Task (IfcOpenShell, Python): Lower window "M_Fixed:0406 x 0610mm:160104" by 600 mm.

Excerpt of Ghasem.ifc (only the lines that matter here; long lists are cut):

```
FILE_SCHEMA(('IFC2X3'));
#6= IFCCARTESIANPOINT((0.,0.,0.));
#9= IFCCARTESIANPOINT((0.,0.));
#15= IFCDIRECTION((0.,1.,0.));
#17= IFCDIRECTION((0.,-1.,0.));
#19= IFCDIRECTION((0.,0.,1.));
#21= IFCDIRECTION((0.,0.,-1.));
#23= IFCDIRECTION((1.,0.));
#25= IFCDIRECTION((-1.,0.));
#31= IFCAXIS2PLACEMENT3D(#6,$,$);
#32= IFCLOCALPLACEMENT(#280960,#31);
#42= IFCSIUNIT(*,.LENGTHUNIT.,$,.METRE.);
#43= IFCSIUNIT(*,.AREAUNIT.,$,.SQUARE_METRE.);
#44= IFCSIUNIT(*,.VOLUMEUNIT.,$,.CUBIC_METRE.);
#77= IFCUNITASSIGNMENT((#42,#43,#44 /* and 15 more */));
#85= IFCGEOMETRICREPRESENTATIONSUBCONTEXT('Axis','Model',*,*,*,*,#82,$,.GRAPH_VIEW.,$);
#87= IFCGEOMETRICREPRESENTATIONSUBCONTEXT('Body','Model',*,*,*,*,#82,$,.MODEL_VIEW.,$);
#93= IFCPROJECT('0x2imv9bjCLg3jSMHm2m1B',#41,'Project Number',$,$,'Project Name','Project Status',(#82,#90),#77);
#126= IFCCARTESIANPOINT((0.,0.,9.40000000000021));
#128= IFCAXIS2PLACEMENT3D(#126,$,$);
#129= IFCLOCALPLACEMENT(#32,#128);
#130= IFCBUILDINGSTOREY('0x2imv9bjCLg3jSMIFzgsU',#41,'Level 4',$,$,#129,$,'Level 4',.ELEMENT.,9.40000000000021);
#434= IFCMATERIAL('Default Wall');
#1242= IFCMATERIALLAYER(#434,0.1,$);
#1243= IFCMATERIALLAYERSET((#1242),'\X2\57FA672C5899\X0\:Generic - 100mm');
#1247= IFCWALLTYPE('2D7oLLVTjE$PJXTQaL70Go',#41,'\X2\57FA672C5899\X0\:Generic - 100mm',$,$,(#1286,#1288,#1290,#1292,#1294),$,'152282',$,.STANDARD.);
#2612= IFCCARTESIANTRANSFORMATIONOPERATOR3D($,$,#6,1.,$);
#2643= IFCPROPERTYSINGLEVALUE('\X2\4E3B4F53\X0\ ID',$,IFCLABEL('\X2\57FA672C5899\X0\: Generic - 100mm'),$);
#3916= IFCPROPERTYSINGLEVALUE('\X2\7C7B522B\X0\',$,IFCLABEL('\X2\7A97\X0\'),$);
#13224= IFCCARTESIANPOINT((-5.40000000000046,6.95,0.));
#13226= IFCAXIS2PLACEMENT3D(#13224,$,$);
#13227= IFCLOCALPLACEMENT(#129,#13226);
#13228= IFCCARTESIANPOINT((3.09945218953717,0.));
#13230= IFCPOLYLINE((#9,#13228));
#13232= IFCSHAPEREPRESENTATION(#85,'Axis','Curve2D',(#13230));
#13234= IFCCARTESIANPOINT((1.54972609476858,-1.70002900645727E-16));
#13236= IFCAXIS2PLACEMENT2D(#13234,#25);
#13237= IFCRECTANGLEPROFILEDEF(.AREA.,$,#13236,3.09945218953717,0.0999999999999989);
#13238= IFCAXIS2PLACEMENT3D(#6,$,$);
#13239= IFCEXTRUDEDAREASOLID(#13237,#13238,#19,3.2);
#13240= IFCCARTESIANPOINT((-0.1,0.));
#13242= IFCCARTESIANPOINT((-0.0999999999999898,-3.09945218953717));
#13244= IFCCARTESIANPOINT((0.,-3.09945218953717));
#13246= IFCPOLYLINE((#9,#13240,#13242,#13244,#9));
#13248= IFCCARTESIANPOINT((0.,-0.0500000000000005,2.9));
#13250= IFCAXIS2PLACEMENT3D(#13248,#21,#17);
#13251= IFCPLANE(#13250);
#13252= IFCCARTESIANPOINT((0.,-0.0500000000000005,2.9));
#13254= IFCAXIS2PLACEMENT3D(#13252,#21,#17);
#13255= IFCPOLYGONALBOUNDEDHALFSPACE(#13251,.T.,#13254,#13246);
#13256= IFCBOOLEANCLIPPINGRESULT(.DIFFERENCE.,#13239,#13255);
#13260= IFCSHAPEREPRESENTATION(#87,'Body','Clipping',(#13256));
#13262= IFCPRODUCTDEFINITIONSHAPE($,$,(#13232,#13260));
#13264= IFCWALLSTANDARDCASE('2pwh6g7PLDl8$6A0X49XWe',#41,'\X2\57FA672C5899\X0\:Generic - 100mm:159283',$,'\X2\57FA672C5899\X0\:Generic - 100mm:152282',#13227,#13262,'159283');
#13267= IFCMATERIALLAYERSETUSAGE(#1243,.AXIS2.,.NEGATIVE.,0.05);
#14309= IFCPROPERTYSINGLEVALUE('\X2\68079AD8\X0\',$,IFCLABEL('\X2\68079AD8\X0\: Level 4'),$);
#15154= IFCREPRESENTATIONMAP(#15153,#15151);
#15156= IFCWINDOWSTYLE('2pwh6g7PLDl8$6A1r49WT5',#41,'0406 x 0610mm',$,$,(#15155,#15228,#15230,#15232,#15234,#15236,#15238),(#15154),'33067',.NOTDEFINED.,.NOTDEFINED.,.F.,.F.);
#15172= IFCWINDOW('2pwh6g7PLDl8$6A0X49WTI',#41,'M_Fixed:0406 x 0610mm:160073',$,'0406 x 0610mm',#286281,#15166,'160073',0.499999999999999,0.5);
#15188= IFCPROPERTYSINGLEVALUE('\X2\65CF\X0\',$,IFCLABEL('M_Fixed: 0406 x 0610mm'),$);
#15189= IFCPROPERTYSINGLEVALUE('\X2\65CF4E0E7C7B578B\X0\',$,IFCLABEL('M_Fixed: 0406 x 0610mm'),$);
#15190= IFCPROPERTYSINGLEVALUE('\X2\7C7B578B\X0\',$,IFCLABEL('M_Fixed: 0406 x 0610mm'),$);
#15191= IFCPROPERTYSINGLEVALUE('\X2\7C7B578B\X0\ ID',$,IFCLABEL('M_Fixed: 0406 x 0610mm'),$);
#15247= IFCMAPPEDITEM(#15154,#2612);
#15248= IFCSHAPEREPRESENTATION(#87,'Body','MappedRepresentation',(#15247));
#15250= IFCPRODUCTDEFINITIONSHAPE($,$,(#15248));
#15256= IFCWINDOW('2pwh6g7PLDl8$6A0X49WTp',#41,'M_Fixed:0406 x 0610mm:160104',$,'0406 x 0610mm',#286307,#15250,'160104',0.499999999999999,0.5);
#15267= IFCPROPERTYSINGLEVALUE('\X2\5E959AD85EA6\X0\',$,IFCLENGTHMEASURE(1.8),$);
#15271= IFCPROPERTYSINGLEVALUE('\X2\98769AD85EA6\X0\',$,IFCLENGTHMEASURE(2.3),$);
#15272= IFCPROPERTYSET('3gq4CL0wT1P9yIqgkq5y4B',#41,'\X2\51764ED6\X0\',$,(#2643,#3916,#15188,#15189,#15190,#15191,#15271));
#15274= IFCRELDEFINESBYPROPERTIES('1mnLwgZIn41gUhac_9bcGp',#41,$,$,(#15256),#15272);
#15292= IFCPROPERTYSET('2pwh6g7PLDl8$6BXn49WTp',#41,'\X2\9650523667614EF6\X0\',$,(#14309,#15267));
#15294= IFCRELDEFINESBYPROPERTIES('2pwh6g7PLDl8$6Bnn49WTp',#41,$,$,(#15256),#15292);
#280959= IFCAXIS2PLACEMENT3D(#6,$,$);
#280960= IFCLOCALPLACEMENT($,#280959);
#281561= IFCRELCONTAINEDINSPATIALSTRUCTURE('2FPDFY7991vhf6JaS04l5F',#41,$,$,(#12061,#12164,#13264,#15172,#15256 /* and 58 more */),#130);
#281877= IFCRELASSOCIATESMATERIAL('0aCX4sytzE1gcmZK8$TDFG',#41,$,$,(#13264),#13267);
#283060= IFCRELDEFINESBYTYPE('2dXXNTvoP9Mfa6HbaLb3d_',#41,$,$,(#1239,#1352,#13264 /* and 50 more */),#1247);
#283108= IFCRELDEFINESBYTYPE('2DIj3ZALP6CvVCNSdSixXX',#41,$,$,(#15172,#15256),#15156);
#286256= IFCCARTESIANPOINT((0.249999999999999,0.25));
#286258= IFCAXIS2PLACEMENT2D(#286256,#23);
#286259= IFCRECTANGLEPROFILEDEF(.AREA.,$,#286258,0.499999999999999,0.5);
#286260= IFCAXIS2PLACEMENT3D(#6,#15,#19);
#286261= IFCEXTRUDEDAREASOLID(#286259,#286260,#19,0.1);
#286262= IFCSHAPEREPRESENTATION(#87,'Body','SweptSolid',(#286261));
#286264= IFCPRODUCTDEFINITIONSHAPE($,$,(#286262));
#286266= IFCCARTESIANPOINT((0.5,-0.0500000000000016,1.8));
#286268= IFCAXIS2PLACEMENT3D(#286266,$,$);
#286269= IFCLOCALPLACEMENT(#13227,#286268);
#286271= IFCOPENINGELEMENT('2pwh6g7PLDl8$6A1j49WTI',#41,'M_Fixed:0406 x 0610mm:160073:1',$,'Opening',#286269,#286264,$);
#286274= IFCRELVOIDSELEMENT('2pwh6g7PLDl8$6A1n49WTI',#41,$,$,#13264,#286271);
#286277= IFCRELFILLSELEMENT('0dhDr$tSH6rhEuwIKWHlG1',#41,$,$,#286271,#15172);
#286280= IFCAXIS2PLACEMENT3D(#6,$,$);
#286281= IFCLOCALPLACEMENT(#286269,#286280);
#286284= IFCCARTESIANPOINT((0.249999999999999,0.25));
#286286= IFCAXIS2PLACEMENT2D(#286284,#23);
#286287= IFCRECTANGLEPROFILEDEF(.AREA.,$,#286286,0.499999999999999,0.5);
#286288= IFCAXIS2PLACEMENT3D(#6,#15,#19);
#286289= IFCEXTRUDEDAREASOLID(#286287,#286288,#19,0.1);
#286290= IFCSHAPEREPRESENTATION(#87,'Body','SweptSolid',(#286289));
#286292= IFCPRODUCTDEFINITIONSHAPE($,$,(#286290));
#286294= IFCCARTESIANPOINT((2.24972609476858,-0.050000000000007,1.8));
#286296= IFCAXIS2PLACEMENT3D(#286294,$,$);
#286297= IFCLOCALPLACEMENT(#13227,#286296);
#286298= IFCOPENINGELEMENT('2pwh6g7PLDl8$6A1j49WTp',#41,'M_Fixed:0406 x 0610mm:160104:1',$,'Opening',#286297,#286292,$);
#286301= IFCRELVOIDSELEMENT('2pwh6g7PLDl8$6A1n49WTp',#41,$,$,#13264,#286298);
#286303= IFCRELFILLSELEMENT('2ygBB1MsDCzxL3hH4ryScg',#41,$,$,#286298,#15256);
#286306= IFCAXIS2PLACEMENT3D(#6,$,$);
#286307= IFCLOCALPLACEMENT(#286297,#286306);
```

```python
import numpy as np
import ifcopenshell
import ifcopenshell.api.geometry
import ifcopenshell.api.pset
import ifcopenshell.util.element
import ifcopenshell.util.placement
import ifcopenshell.util.unit

model = ifcopenshell.open("Ghasem.ifc")
unit_scale = ifcopenshell.util.unit.calculate_unit_scale(model)

window = model.by_guid("2pwh6g7PLDl8$6A0X49WTp")
opening = window.FillsVoids[0].RelatingOpeningElement
dz = -0.6 / unit_scale

shift = np.array([0.0, 0.0, dz])
# The window is placed relative to its opening, so it follows when the opening moves.
matrix = ifcopenshell.util.placement.get_local_placement(opening.ObjectPlacement)
matrix[:3, 3] += shift
ifcopenshell.api.geometry.edit_object_placement(
    model, product=opening, matrix=matrix, is_si=False, should_transform_children=True
)

# Keep the stored heights in step.
pset = model.by_id(ifcopenshell.util.element.get_pset(window, "其他", should_inherit=False)["id"])
ifcopenshell.api.pset.edit_pset(model, pset=pset, properties={
    "顶高度": model.create_entity("IfcLengthMeasure", ifcopenshell.util.element.get_pset(window, "其他", "顶高度") + dz),
})
pset = model.by_id(ifcopenshell.util.element.get_pset(window, "限制条件", should_inherit=False)["id"])
ifcopenshell.api.pset.edit_pset(model, pset=pset, properties={
    "底高度": model.create_entity("IfcLengthMeasure", ifcopenshell.util.element.get_pset(window, "限制条件", "底高度") + dz),
})

print(f"moved by {dz * unit_scale:+.3f} m")

model.write("Ghasem-out.ifc")
```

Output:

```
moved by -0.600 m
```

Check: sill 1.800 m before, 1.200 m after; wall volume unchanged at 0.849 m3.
